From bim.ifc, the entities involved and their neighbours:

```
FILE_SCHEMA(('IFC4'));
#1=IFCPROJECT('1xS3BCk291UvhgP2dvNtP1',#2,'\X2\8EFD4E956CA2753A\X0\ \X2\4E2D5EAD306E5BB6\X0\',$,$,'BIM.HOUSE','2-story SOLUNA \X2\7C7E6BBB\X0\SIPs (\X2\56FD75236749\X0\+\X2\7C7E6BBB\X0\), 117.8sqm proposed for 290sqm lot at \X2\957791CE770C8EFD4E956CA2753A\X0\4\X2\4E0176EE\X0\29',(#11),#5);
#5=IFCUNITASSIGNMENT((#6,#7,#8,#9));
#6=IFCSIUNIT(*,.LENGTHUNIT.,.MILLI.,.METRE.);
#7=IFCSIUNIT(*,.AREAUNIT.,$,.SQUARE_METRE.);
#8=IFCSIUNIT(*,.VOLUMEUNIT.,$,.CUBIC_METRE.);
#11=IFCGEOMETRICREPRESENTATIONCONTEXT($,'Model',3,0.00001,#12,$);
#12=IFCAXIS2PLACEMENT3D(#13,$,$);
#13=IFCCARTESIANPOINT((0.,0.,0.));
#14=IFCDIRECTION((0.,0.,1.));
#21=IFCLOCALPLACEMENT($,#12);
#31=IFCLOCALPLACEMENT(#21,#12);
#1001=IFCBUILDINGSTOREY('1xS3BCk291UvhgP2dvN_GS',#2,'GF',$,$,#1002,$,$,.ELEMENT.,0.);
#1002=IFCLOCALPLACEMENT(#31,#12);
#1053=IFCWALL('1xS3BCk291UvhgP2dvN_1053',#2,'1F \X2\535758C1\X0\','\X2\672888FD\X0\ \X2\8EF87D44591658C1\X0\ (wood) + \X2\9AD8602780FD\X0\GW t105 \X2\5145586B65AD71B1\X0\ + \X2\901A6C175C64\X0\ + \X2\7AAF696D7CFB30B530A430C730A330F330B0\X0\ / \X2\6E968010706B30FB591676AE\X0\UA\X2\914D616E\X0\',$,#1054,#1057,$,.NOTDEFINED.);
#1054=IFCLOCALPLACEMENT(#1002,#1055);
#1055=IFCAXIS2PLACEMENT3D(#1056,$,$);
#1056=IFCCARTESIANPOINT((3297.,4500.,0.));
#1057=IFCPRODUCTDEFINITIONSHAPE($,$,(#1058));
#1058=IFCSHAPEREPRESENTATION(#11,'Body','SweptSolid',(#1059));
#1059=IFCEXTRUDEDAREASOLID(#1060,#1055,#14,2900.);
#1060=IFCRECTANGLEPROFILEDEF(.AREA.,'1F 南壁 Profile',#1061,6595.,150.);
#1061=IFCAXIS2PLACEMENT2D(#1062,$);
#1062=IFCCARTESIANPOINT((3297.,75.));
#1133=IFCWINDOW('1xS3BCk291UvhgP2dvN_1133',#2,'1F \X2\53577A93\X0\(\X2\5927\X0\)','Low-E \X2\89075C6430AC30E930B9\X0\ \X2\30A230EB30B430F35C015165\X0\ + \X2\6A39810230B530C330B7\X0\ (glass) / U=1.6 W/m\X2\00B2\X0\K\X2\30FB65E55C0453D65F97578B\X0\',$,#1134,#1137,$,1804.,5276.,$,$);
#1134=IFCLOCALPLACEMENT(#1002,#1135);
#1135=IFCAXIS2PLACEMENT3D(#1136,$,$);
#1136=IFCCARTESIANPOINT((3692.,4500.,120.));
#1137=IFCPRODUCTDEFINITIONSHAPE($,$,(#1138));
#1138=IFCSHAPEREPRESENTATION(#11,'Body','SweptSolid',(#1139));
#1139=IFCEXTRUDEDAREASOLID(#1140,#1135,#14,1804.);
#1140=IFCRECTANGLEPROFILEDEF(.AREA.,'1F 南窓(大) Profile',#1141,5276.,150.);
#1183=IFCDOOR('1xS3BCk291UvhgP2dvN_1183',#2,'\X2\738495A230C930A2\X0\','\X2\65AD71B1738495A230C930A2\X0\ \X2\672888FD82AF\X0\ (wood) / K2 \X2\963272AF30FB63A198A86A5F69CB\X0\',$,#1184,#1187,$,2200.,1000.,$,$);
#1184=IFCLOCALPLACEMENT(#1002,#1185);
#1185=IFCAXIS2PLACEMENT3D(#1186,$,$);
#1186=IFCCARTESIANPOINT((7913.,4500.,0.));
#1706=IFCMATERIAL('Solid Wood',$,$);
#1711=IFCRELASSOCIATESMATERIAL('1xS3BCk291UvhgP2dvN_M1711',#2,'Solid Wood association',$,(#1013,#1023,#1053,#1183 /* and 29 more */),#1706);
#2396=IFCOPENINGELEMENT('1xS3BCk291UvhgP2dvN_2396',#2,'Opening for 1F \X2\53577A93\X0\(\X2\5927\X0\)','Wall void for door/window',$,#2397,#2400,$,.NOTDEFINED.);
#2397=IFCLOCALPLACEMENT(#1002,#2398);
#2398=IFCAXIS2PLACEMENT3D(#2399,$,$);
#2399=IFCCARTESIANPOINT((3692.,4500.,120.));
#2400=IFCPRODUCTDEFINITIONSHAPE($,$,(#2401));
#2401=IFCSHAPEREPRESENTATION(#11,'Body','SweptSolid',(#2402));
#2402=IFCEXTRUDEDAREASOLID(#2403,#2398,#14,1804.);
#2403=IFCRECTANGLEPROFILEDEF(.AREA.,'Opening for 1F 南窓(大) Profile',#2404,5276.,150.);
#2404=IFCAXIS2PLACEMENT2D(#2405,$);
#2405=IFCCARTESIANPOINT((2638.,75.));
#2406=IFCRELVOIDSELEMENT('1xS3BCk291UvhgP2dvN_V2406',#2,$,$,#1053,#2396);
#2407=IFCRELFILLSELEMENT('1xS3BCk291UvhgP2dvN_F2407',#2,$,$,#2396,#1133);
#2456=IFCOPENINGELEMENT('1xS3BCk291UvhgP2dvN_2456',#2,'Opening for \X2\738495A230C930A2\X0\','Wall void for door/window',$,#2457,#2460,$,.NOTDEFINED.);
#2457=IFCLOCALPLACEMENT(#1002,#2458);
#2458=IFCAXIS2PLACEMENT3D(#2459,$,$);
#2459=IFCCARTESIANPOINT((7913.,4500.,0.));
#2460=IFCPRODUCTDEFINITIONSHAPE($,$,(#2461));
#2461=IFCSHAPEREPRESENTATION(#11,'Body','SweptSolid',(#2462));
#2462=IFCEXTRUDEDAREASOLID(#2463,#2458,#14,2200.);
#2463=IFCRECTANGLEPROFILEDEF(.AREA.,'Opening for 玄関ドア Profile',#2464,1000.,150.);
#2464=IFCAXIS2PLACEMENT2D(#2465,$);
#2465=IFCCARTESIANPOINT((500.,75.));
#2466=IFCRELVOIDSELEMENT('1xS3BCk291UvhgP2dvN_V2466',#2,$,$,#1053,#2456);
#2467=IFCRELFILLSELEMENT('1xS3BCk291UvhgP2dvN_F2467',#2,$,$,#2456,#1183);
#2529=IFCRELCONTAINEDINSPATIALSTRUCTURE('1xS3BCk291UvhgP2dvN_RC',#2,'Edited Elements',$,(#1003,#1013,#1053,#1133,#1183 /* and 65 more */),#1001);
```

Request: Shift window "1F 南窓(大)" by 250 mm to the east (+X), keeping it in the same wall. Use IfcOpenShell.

```python
import ifcopenshell
import ifcopenshell.api.geometry
import ifcopenshell.util.placement

model = ifcopenshell.open("bim.ifc")

window = model.by_guid("1xS3BCk291UvhgP2dvN_1133")
opening = window.FillsVoids[0].RelatingOpeningElement
wall = opening.VoidsElements[0].RelatingBuildingElement

wall_matrix = ifcopenshell.util.placement.get_local_placement(wall.ObjectPlacement)
shift = wall_matrix[:3, 0] * 250.0
before = ifcopenshell.util.placement.get_local_placement(window.ObjectPlacement)[:3, 3].copy()

# The window is not placed relative to its opening, so move both.
for product in (opening, window):
    matrix = ifcopenshell.util.placement.get_local_placement(product.ObjectPlacement)
    matrix[:3, 3] += shift
    ifcopenshell.api.geometry.edit_object_placement(model, product=product, matrix=matrix, is_si=False)

after = ifcopenshell.util.placement.get_local_placement(window.ObjectPlacement)[:3, 3]
print("window moved by", (after - before).round(3) + 0.0)

model.write("bim_updated.ifc")
```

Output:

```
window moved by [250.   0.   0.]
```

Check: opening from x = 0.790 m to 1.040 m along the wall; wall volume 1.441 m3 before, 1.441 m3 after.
